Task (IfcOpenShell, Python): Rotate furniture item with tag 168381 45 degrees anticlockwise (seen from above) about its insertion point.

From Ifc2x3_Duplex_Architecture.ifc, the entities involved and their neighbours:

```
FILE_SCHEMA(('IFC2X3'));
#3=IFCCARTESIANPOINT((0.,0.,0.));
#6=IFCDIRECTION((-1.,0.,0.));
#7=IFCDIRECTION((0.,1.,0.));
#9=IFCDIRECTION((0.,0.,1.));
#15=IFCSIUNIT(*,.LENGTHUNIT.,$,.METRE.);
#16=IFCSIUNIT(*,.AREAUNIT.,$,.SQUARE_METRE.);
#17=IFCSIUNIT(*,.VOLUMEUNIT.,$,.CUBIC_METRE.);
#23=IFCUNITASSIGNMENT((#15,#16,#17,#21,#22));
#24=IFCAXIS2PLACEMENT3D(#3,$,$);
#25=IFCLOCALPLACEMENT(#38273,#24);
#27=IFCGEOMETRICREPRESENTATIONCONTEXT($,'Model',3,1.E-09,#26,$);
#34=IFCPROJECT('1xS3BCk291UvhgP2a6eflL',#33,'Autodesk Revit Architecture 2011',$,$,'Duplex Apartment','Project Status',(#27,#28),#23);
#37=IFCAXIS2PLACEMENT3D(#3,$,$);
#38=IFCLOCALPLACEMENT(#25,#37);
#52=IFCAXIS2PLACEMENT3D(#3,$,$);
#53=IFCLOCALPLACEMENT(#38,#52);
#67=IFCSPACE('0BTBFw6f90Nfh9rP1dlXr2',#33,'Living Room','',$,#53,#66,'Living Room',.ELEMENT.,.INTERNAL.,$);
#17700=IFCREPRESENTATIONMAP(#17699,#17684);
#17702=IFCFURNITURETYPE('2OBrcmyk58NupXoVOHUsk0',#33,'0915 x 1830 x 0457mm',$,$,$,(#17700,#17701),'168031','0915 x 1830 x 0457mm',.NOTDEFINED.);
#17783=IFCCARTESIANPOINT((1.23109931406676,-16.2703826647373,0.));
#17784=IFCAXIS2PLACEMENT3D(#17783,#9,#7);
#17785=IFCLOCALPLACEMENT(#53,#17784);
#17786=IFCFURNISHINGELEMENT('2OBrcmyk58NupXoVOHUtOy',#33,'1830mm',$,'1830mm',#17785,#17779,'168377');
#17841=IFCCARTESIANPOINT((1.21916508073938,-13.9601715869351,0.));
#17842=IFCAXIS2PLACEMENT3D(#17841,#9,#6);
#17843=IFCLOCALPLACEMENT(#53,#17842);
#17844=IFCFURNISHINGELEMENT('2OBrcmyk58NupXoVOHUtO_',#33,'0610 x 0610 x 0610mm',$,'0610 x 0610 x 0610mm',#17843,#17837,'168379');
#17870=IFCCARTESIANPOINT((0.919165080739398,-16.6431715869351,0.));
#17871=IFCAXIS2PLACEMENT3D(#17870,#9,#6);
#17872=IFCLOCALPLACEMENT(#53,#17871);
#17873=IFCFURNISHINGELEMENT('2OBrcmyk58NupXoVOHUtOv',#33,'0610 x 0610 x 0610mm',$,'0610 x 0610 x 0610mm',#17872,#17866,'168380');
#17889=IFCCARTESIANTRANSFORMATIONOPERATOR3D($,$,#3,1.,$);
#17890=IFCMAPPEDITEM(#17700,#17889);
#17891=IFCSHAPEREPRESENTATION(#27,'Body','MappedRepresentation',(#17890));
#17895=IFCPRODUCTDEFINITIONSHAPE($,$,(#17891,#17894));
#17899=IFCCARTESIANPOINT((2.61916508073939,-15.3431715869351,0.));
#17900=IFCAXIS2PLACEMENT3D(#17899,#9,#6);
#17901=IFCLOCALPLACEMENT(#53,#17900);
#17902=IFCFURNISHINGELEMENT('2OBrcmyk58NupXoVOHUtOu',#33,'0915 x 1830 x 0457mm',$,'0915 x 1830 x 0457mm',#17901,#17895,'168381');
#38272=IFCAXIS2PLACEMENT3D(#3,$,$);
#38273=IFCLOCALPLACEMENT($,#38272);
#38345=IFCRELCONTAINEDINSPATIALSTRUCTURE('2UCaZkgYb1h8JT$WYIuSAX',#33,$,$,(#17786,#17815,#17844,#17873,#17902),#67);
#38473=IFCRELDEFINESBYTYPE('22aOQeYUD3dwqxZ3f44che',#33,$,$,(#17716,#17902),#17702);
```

```python
import ifcopenshell
import ifcopenshell.api.geometry
import ifcopenshell.util.placement

model = ifcopenshell.open("Ifc2x3_Duplex_Architecture.ifc")

item = model.by_guid("2OBrcmyk58NupXoVOHUtOu")
matrix = ifcopenshell.util.placement.get_local_placement(item.ObjectPlacement)
matrix = matrix @ ifcopenshell.util.placement.rotation(45, "Z")
ifcopenshell.api.geometry.edit_object_placement(model, product=item, matrix=matrix, is_si=False)

print(ifcopenshell.util.placement.get_local_placement(item.ObjectPlacement).round(3) + 0.0)

model.write("Ifc2x3_Duplex_Architecture-out.ifc")
```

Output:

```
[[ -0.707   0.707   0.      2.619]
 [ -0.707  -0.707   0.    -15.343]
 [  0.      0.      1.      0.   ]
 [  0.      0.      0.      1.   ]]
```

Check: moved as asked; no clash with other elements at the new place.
